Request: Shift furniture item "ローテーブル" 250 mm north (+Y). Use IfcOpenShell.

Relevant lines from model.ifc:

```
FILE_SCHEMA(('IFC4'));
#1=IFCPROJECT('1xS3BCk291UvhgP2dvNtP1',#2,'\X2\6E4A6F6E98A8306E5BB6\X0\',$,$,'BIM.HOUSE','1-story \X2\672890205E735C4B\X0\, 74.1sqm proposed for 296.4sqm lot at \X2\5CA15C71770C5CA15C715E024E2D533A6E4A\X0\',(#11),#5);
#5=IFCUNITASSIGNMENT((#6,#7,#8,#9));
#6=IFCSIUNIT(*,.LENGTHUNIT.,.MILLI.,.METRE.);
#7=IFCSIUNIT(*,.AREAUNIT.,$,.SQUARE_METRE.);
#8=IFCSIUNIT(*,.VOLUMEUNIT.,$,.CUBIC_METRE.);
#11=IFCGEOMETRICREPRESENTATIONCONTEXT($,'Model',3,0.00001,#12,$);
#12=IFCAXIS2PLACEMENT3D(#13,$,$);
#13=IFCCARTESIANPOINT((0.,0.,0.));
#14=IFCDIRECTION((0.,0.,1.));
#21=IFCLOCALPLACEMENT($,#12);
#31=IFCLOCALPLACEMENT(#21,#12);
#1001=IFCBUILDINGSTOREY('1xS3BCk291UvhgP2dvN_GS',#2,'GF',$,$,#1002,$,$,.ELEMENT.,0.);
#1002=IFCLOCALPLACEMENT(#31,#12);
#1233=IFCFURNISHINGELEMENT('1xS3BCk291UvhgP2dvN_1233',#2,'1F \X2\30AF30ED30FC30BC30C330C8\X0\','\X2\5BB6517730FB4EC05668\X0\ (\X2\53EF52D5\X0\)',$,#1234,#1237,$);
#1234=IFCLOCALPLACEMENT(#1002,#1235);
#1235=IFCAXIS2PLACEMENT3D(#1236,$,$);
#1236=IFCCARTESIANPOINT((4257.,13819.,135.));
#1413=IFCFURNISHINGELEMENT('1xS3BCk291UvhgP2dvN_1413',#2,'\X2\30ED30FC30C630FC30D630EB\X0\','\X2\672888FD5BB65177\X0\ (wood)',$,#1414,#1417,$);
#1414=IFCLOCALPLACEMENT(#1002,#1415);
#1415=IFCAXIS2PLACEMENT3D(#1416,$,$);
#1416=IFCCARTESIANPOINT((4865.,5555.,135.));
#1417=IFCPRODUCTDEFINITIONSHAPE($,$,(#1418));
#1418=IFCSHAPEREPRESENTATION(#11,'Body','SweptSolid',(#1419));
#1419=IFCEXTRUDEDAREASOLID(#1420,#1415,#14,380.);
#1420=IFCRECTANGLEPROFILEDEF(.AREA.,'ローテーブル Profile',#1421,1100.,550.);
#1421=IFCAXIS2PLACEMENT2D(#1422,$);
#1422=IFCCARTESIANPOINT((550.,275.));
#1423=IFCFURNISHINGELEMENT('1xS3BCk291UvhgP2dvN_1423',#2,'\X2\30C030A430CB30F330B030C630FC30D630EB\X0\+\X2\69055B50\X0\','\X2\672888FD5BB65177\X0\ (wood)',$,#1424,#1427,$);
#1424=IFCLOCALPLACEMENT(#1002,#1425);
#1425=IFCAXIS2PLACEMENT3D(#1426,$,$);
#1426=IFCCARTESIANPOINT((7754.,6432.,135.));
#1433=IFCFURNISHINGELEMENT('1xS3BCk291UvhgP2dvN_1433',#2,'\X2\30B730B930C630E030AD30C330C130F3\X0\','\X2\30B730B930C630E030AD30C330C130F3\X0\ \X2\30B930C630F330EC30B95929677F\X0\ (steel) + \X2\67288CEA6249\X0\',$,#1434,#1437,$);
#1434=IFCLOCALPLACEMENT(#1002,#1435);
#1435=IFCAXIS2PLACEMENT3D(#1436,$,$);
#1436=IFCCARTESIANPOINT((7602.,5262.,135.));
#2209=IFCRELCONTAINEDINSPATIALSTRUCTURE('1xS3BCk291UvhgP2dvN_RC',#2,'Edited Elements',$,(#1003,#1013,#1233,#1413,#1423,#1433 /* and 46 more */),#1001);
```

```python
import ifcopenshell
import ifcopenshell.api.geometry
import ifcopenshell.util.placement
import ifcopenshell.util.unit

model = ifcopenshell.open("model.ifc")
unit_scale = ifcopenshell.util.unit.calculate_unit_scale(model)

item = model.by_guid("1xS3BCk291UvhgP2dvN_1413")
matrix = ifcopenshell.util.placement.get_local_placement(item.ObjectPlacement)
matrix[1, 3] += 0.25 / unit_scale
ifcopenshell.api.geometry.edit_object_placement(model, product=item, matrix=matrix, is_si=False)

print(ifcopenshell.util.placement.get_local_placement(item.ObjectPlacement).round(3) + 0.0)

model.write("model_rev.ifc")
```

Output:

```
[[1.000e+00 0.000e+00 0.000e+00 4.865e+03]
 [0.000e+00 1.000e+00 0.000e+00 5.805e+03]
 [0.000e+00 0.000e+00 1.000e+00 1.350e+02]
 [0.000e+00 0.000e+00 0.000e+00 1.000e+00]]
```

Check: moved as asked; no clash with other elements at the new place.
